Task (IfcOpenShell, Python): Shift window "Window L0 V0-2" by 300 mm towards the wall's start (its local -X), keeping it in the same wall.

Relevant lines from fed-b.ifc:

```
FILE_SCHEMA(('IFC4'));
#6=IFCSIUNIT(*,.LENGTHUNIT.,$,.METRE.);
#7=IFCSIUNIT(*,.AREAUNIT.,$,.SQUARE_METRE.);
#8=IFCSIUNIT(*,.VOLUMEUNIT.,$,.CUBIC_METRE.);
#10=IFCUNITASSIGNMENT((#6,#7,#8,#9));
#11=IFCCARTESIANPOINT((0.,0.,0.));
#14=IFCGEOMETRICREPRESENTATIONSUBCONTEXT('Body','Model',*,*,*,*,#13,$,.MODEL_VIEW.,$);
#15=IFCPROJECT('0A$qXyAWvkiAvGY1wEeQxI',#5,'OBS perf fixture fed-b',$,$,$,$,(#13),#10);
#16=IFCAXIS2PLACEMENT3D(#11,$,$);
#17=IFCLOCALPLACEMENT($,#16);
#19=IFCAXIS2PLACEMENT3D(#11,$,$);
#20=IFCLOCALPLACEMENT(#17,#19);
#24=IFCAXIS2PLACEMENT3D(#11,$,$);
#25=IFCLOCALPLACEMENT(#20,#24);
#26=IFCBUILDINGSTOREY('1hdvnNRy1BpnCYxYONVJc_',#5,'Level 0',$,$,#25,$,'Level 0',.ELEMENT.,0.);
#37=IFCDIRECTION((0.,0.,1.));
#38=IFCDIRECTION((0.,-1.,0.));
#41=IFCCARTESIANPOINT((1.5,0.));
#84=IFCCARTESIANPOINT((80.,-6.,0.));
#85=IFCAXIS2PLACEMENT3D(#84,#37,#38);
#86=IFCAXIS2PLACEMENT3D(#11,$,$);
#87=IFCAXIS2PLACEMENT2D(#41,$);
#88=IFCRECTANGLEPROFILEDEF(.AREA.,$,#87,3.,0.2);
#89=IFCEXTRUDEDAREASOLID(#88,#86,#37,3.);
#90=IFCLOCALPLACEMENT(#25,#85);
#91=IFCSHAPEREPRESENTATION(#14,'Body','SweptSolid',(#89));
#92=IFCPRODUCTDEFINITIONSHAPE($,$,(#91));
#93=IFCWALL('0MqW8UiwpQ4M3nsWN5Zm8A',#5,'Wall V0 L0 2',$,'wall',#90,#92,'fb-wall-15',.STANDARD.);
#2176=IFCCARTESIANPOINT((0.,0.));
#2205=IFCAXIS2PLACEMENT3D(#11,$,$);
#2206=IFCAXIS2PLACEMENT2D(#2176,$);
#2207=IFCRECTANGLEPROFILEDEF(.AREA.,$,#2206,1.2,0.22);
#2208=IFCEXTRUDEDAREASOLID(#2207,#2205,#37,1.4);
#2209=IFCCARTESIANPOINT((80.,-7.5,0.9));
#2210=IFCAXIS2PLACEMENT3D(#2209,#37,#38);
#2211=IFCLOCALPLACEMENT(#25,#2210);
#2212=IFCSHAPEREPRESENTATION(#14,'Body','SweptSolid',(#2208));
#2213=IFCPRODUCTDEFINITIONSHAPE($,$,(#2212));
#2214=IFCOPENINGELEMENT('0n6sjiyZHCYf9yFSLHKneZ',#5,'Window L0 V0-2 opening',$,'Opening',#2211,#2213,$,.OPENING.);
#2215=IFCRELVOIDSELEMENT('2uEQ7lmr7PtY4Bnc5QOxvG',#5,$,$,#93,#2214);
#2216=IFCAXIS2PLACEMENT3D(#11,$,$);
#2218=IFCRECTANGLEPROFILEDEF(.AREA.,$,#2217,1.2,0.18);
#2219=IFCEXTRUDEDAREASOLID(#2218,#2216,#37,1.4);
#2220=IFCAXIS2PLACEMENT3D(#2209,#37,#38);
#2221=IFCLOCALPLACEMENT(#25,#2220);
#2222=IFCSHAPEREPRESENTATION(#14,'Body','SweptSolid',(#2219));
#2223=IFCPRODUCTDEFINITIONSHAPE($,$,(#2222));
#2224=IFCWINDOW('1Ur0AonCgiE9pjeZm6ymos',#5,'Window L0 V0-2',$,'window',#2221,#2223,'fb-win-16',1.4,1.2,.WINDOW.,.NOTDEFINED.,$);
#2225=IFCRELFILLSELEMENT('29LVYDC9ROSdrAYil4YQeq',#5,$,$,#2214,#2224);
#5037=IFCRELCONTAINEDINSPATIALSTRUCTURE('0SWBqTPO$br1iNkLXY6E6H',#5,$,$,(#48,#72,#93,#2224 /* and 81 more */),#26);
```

```python
import ifcopenshell
import ifcopenshell.api.geometry
import ifcopenshell.util.placement
import ifcopenshell.util.unit

model = ifcopenshell.open("fed-b.ifc")
unit_scale = ifcopenshell.util.unit.calculate_unit_scale(model)

window = model.by_guid("1Ur0AonCgiE9pjeZm6ymos")
opening = window.FillsVoids[0].RelatingOpeningElement
wall = opening.VoidsElements[0].RelatingBuildingElement

wall_matrix = ifcopenshell.util.placement.get_local_placement(wall.ObjectPlacement)
shift = wall_matrix[:3, 0] * -0.3 / unit_scale
before = ifcopenshell.util.placement.get_local_placement(window.ObjectPlacement)[:3, 3].copy()

# The window is not placed relative to its opening, so move both.
for product in (opening, window):
    matrix = ifcopenshell.util.placement.get_local_placement(product.ObjectPlacement)
    matrix[:3, 3] += shift
    ifcopenshell.api.geometry.edit_object_placement(model, product=product, matrix=matrix, is_si=False)

after = ifcopenshell.util.placement.get_local_placement(window.ObjectPlacement)[:3, 3]
print("window moved by", (after - before).round(3) + 0.0)

model.write("fed-b_rev.ifc")
```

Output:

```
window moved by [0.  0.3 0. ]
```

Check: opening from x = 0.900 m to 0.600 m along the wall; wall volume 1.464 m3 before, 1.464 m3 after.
